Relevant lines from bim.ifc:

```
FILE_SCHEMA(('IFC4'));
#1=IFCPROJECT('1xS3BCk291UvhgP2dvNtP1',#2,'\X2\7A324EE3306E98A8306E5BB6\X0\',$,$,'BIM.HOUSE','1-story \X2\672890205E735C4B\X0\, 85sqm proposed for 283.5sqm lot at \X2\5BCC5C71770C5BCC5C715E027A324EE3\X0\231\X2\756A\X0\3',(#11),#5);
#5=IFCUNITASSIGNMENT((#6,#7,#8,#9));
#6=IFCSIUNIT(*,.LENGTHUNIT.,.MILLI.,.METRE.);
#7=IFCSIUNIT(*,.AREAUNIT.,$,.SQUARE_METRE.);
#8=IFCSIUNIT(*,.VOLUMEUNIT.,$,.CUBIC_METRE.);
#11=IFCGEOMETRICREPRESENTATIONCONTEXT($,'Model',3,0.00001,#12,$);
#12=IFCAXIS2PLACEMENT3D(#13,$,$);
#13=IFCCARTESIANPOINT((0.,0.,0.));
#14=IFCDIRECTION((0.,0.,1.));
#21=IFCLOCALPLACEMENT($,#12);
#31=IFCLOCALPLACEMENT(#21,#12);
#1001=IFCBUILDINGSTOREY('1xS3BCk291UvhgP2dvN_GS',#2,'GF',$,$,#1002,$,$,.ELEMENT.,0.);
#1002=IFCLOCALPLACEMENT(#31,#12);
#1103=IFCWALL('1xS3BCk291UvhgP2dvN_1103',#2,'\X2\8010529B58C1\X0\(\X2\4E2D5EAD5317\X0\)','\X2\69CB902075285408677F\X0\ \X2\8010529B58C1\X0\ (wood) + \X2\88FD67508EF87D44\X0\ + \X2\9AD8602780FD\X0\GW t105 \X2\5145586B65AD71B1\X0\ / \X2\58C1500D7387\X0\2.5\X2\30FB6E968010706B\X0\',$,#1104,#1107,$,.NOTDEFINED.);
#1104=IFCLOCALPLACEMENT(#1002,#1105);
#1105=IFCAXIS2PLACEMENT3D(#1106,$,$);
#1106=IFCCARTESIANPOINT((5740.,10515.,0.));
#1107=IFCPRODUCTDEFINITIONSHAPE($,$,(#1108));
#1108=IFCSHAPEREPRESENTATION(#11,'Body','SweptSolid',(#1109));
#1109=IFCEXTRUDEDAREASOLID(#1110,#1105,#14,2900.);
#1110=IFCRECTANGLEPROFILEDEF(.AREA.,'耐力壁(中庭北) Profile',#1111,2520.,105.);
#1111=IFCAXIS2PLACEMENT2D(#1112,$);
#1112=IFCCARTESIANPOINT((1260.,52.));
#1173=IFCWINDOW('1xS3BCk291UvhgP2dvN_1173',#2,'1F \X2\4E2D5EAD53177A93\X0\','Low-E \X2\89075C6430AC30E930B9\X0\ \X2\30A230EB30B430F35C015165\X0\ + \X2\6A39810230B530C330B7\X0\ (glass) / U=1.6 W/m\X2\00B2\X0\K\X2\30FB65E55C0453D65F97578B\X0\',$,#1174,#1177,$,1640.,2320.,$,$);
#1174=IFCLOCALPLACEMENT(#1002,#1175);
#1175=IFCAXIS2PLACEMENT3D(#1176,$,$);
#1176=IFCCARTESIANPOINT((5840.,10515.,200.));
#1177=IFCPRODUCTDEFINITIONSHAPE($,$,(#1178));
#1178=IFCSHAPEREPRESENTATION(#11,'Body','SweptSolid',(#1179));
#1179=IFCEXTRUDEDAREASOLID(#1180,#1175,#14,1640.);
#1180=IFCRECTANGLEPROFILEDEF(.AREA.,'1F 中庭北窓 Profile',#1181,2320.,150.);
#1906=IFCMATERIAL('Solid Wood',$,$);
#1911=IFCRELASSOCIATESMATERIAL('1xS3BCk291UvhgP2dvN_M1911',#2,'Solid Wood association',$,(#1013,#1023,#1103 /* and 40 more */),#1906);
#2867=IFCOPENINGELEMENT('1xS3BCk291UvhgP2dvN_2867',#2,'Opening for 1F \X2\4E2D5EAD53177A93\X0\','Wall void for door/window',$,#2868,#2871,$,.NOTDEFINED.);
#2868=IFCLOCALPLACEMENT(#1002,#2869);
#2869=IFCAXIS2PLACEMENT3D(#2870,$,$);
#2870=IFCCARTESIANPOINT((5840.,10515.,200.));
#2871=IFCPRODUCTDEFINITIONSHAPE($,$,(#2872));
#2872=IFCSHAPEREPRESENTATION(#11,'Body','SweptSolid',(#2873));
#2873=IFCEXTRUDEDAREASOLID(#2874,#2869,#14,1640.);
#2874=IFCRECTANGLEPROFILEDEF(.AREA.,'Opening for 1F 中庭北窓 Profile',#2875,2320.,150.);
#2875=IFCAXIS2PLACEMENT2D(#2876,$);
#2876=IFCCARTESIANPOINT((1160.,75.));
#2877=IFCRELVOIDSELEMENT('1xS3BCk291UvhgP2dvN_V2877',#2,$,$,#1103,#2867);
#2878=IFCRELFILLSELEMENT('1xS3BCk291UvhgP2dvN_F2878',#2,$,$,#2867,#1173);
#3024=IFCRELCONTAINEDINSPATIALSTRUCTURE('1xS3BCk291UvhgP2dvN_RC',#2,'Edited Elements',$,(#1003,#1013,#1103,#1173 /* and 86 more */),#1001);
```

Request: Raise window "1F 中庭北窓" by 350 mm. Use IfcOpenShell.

```python
import numpy as np
import ifcopenshell
import ifcopenshell.api.geometry
import ifcopenshell.util.placement
import ifcopenshell.util.unit

model = ifcopenshell.open("bim.ifc")
unit_scale = ifcopenshell.util.unit.calculate_unit_scale(model)

window = model.by_guid("1xS3BCk291UvhgP2dvN_1173")
opening = window.FillsVoids[0].RelatingOpeningElement
dz = 350.0

shift = np.array([0.0, 0.0, dz])
# The window is not placed relative to its opening, so move both.
for product in (opening, window):
    matrix = ifcopenshell.util.placement.get_local_placement(product.ObjectPlacement)
    matrix[:3, 3] += shift
    ifcopenshell.api.geometry.edit_object_placement(model, product=product, matrix=matrix, is_si=False)

print(f"moved by {dz * unit_scale:+.3f} m")

model.write("bim_rev.ifc")
```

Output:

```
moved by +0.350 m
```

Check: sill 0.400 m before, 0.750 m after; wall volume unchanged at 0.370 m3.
